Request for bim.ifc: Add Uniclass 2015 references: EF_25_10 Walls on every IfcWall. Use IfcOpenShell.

First a look at what the model holds.

```python
import ifcopenshell

model = ifcopenshell.open("bim.ifc")
print(model.schema)
print("classifications:", [c.Name for c in model.by_type("IfcClassification")])
for ifc_class in ("IfcDoor", "IfcRoof", "IfcStair", "IfcWall", "IfcWindow"):
    print(ifc_class, len(model.by_type(ifc_class)))
```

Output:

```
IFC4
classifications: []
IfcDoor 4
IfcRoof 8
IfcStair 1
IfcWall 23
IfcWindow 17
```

```python
import ifcopenshell
import ifcopenshell.api.classification

model = ifcopenshell.open("bim.ifc")

system = ifcopenshell.api.classification.add_classification(model, classification="Uniclass 2015")

codes = {
    "IfcWall": ("EF_25_10", "Walls"),
}
for ifc_class, (code, name) in codes.items():
    products = model.by_type(ifc_class)
    ifcopenshell.api.classification.add_reference(
        model, products=products, classification=system, identification=code, name=name
    )
    print(code, len(products))

model.write("bim_updated.ifc")
```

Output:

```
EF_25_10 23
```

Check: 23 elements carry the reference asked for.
